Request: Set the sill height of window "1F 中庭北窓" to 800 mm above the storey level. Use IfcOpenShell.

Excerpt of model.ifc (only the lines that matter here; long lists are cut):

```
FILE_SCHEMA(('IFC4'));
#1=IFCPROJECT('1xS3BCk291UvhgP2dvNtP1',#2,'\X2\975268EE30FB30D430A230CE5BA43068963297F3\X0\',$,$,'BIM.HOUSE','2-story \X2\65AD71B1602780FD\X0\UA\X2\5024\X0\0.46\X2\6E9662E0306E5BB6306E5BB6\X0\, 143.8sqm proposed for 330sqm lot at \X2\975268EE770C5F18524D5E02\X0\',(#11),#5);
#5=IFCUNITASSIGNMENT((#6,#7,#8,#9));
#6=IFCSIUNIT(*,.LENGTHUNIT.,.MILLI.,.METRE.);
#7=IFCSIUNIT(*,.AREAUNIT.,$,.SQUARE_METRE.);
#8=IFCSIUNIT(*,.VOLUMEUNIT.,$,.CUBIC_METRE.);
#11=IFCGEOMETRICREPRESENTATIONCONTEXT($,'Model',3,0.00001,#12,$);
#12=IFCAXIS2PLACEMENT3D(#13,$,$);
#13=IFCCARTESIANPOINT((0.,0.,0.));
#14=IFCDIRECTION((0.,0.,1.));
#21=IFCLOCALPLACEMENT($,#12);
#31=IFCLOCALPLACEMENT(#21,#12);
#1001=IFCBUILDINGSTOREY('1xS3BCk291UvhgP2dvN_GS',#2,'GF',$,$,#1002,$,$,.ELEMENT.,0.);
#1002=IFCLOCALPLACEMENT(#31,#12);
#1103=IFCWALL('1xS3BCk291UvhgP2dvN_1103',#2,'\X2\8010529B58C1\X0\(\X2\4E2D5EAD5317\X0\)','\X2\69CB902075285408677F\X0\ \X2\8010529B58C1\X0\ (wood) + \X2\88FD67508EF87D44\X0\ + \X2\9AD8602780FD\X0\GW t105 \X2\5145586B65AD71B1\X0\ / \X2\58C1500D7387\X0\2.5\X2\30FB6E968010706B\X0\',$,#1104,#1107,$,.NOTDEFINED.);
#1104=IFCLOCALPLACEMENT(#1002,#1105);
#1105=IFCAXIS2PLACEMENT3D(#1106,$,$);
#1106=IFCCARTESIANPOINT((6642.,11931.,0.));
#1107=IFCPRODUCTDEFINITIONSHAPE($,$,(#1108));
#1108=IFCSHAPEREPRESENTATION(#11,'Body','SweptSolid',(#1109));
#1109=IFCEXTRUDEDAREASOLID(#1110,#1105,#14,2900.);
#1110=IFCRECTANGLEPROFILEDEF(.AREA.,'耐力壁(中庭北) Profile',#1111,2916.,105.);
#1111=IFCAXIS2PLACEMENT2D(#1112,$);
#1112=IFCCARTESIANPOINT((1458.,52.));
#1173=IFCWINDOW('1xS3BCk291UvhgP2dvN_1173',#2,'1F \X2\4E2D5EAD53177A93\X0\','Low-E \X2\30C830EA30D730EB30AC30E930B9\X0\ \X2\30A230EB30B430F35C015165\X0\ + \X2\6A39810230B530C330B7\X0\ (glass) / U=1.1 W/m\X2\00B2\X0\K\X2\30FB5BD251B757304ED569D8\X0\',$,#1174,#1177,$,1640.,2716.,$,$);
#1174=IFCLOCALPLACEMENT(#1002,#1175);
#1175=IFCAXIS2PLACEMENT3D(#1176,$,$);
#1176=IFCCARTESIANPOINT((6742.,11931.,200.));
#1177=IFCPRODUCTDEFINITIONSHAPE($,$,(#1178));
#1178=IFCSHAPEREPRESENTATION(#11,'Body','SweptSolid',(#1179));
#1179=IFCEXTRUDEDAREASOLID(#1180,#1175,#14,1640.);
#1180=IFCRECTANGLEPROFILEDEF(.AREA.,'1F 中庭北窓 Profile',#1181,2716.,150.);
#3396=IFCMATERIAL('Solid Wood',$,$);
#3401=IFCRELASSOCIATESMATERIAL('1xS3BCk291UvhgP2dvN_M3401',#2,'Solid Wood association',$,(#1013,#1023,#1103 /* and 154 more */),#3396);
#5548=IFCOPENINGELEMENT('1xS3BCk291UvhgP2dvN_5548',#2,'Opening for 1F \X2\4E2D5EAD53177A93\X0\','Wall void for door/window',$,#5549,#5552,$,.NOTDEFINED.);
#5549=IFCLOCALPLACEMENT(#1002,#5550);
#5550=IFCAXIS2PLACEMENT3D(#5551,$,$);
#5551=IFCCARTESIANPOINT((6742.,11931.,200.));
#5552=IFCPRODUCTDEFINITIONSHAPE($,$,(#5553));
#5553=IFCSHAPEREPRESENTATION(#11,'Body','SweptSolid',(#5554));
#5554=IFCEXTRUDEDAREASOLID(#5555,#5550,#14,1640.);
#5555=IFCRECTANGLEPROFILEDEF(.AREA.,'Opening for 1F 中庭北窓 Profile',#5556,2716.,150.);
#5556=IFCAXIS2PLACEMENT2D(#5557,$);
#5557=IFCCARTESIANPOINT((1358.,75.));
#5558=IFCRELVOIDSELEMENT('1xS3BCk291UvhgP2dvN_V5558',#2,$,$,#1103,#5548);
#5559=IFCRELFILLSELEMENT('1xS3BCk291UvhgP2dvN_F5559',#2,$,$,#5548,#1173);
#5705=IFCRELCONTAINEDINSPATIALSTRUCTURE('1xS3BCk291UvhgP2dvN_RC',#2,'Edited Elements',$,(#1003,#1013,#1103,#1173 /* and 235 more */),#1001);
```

```python
import numpy as np
import ifcopenshell
import ifcopenshell.api.geometry
import ifcopenshell.geom
import ifcopenshell.util.element
import ifcopenshell.util.placement
import ifcopenshell.util.shape
import ifcopenshell.util.unit

model = ifcopenshell.open("model.ifc")
unit_scale = ifcopenshell.util.unit.calculate_unit_scale(model)

window = model.by_guid("1xS3BCk291UvhgP2dvN_1173")
opening = window.FillsVoids[0].RelatingOpeningElement
storey = ifcopenshell.util.element.get_container(window, ifc_class="IfcBuildingStorey")
level = ifcopenshell.util.placement.get_local_placement(storey.ObjectPlacement)[2, 3]

# The opening's origin need not be at the sill, so measure its lowest point.
shape = ifcopenshell.geom.create_shape(ifcopenshell.geom.settings(), opening)
bottom = ifcopenshell.util.shape.get_shape_bottom_elevation(shape, shape.geometry) / unit_scale
dz = level + 0.8 / unit_scale - bottom

shift = np.array([0.0, 0.0, dz])
# The window is not placed relative to its opening, so move both.
for product in (opening, window):
    matrix = ifcopenshell.util.placement.get_local_placement(product.ObjectPlacement)
    matrix[:3, 3] += shift
    ifcopenshell.api.geometry.edit_object_placement(model, product=product, matrix=matrix, is_si=False)

print(f"moved by {dz * unit_scale:+.3f} m")

model.write("model-out.ifc")
```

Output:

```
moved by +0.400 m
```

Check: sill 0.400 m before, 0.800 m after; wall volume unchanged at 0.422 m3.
